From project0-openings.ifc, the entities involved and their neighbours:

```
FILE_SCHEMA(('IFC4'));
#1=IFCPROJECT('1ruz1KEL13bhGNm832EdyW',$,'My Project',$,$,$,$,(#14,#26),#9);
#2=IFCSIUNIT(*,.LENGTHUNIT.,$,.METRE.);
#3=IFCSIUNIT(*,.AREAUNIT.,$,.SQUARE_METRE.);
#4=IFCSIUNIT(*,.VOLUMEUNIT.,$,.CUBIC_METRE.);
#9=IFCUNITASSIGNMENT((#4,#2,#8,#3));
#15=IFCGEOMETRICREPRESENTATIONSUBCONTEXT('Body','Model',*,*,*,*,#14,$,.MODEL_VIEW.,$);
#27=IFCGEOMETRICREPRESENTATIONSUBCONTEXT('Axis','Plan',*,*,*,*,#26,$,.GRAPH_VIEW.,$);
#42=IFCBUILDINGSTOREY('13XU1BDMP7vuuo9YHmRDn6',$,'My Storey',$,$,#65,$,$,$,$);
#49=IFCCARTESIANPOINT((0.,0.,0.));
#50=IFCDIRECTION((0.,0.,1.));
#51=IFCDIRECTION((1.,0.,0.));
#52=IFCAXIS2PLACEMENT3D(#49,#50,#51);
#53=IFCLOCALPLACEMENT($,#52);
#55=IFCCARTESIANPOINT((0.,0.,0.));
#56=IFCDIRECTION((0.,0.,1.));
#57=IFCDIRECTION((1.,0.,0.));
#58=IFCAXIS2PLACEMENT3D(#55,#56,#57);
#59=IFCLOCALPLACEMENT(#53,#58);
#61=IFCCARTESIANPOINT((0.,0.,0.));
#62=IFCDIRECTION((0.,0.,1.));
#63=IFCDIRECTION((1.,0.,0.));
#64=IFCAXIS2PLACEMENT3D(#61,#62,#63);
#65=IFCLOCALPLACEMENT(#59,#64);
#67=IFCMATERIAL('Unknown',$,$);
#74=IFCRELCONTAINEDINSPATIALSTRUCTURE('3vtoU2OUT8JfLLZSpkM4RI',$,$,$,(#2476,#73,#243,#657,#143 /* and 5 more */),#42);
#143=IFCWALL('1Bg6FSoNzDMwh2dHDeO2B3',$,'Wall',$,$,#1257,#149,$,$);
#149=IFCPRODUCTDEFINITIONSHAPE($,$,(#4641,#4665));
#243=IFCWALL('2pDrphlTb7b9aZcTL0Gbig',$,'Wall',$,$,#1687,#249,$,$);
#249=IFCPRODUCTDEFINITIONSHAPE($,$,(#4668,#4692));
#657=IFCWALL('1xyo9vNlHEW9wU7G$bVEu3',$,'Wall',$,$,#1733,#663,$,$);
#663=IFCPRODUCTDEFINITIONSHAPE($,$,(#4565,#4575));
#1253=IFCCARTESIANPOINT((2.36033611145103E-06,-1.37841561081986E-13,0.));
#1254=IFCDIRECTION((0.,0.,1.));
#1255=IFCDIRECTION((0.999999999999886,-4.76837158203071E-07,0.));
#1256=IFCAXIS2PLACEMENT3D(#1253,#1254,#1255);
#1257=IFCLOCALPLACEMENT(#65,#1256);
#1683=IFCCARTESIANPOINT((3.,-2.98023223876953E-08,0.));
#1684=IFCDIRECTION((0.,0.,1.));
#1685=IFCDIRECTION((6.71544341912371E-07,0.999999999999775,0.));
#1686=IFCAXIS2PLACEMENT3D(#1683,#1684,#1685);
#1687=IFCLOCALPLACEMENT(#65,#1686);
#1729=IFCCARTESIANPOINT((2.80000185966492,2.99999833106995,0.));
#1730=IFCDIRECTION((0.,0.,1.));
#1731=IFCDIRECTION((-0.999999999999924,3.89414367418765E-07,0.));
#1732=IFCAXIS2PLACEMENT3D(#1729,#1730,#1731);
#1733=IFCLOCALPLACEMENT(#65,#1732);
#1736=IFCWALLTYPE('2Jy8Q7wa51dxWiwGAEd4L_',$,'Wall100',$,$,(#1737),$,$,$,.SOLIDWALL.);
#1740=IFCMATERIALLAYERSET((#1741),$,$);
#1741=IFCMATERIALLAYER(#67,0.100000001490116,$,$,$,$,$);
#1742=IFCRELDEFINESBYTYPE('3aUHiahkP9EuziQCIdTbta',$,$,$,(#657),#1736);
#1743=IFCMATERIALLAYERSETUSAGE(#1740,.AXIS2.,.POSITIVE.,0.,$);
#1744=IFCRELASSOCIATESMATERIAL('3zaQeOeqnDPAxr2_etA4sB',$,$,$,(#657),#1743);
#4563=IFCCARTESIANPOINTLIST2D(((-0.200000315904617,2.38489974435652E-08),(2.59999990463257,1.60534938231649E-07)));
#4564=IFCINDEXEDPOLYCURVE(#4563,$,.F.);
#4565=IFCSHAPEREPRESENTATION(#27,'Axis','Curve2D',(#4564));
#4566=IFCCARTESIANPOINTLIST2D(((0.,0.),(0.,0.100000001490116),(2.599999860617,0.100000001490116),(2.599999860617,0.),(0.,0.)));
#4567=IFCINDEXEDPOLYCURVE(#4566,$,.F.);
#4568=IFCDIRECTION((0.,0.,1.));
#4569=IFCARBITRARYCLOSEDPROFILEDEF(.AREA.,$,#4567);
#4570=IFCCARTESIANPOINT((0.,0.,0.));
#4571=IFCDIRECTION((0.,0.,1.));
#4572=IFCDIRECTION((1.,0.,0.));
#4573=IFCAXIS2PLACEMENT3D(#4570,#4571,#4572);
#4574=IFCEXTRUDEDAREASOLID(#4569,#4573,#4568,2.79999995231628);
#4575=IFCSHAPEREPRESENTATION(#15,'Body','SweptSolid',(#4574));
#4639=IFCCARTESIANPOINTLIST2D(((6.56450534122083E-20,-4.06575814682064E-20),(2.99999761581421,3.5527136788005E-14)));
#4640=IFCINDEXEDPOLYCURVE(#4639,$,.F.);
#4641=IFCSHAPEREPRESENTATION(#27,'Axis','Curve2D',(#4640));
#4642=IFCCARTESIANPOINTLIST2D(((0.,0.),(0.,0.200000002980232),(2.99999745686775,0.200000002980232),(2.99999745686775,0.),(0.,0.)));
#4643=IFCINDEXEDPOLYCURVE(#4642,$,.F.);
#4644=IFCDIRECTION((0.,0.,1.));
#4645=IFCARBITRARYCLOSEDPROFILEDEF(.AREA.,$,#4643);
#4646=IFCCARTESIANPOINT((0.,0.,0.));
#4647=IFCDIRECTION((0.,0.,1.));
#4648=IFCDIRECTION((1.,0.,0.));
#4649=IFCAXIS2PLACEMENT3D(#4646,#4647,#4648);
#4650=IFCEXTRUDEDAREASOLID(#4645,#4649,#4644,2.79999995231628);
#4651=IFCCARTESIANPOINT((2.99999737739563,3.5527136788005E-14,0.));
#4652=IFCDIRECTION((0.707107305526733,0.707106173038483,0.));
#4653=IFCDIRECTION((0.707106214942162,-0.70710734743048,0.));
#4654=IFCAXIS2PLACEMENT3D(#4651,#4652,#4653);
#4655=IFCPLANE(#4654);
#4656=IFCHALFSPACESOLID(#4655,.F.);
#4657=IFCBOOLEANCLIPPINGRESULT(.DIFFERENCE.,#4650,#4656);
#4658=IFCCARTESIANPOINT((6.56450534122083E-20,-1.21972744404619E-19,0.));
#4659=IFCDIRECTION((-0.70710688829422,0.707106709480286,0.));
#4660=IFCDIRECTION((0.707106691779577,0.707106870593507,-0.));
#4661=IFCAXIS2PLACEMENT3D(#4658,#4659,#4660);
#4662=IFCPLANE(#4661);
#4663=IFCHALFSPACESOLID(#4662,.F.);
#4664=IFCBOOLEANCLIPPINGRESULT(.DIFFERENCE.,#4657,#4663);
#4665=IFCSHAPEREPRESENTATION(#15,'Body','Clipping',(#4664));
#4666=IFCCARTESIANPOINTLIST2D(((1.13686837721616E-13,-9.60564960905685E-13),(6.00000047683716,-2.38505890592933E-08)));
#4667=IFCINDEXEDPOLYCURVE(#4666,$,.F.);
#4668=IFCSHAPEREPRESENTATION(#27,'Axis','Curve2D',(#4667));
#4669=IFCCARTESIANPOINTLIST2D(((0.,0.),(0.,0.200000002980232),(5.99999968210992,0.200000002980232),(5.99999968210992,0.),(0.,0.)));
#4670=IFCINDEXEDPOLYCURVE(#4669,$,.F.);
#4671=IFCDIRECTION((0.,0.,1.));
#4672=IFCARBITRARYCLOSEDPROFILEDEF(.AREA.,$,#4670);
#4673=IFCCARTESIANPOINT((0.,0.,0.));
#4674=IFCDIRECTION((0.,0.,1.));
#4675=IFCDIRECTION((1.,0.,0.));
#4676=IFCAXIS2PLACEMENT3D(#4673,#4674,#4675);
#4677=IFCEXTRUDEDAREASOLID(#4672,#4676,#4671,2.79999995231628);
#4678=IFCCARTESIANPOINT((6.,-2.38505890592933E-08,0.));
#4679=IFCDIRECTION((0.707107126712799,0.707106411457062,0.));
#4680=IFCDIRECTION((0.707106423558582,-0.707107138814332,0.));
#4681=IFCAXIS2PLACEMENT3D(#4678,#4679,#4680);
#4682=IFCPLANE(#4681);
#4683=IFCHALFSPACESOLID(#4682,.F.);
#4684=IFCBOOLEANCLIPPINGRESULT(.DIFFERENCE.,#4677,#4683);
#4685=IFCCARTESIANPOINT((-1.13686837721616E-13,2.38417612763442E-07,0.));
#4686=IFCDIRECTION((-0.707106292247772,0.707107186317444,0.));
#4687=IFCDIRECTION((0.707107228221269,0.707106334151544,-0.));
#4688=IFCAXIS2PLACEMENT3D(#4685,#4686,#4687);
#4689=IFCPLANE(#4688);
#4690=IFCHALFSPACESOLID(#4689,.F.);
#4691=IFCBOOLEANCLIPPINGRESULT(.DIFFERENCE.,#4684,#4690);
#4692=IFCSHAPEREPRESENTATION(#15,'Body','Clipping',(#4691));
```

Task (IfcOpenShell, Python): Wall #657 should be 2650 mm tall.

```python
import ifcopenshell
import ifcopenshell.geom
import ifcopenshell.util.representation
import ifcopenshell.util.shape

model = ifcopenshell.open("project0-openings.ifc")
settings = ifcopenshell.geom.settings()


def volume(element):
    """Net volume in cubic metres, openings subtracted."""
    shape = ifcopenshell.geom.create_shape(settings, element)
    return ifcopenshell.util.shape.get_volume(shape.geometry)


wall = model.by_id(657)
before = volume(wall)

body = ifcopenshell.util.representation.get_representation(wall, "Model", "Body")
solid = body.Items[0]
old_height = solid.Depth
solid.Depth = 2.65
after = volume(wall)

print(f"height {old_height:g} -> {solid.Depth:g}, volume {before:.3f} -> {after:.3f} m3")

model.write("project0-openings_v2.ifc")
```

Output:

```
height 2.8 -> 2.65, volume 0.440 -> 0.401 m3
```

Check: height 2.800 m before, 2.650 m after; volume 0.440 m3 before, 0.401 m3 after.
